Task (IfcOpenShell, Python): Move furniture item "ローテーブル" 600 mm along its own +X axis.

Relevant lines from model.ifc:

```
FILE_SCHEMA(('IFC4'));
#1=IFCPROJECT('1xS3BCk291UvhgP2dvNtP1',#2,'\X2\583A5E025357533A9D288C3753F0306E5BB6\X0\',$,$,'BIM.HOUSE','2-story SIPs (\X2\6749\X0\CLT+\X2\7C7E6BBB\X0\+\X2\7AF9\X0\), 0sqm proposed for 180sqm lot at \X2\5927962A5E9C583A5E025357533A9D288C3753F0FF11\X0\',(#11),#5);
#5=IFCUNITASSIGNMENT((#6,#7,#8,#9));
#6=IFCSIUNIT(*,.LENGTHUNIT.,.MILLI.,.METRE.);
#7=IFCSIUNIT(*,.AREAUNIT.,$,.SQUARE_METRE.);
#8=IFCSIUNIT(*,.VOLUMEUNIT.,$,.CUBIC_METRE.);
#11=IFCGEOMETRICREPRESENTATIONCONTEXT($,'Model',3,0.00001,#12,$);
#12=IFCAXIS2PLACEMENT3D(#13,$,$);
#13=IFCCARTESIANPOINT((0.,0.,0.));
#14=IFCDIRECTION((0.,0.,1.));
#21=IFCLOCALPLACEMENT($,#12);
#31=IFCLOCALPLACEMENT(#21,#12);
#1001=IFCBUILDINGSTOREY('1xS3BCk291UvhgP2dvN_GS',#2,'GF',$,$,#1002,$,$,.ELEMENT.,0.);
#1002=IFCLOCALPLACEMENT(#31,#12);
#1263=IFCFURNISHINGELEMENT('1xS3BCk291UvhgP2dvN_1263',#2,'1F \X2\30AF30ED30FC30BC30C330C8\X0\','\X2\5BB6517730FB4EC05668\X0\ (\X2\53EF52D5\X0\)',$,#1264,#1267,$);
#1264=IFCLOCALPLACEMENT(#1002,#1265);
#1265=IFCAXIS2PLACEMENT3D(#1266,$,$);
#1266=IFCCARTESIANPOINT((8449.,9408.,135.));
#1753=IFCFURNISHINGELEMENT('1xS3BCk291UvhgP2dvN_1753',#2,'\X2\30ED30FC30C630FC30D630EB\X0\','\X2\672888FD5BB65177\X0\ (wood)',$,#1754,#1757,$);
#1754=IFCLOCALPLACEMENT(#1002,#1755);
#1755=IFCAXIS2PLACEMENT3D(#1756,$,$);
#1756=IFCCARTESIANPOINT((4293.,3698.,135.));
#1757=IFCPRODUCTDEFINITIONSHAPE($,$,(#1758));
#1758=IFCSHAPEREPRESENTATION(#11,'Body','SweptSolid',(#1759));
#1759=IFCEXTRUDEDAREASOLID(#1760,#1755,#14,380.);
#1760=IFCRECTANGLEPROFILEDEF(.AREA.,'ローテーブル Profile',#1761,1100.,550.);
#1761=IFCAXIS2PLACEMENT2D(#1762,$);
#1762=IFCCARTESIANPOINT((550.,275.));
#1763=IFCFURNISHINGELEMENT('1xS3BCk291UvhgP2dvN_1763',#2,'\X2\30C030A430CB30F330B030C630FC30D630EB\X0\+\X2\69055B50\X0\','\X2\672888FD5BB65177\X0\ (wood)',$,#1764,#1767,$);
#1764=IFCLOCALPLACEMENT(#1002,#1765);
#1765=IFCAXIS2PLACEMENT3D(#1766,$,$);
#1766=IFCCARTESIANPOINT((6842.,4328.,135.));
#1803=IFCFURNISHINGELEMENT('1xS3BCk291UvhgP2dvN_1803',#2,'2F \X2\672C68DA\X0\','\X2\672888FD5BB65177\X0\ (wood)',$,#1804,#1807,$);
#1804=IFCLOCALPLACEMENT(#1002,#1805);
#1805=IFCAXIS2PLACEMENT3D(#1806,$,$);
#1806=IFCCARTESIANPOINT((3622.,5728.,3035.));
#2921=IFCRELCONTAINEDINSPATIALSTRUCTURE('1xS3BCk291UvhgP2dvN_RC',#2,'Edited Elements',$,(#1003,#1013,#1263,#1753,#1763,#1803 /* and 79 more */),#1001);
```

```python
import ifcopenshell
import ifcopenshell.api.geometry
import ifcopenshell.util.placement

model = ifcopenshell.open("model.ifc")

item = model.by_guid("1xS3BCk291UvhgP2dvN_1753")
matrix = ifcopenshell.util.placement.get_local_placement(item.ObjectPlacement)
matrix[:3, 3] += matrix[:3, 0] * 600.0
ifcopenshell.api.geometry.edit_object_placement(model, product=item, matrix=matrix, is_si=False)

print(ifcopenshell.util.placement.get_local_placement(item.ObjectPlacement).round(3) + 0.0)

model.write("model_edited.ifc")
```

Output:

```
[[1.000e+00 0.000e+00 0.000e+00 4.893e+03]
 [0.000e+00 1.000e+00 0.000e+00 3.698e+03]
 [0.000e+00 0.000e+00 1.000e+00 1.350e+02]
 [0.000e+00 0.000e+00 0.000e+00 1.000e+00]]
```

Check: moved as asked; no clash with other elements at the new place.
